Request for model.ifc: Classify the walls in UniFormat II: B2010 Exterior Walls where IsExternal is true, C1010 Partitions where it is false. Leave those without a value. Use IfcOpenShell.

First a look at what the model holds.

```python
import ifcopenshell
import ifcopenshell.util.element

model = ifcopenshell.open("model.ifc")
print(model.schema)
print("classifications:", [c.Name for c in model.by_type("IfcClassification")])
values = [ifcopenshell.util.element.get_pset(e, "Pset_WallCommon", "IsExternal") for e in model.by_type("IfcWall")]
for value in (True, False, None):
    print("IsExternal", value, values.count(value))
```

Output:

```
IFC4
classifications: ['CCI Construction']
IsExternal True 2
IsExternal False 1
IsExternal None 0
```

```python
import ifcopenshell
import ifcopenshell.api.classification
import ifcopenshell.util.element

model = ifcopenshell.open("model.ifc")

system = ifcopenshell.api.classification.add_classification(model, classification="UniFormat II")

walls = model.by_type("IfcWall")
external = {e: ifcopenshell.util.element.get_pset(e, "Pset_WallCommon", "IsExternal") for e in walls}
for flag, code, name in ((True, "B2010", "Exterior Walls"), (False, "C1010", "Partitions")):
    products = [e for e in walls if external[e] is flag]
    ifcopenshell.api.classification.add_reference(
        model, products=products, classification=system, identification=code, name=name
    )
    print(code, len(products))

model.write("model_v2.ifc")
```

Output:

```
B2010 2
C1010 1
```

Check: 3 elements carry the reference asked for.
